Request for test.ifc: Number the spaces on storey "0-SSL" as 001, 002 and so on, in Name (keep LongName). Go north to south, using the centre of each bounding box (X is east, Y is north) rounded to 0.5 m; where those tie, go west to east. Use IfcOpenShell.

First a look at what the model holds.

```python
import ifcopenshell
import ifcopenshell.util.element
import ifcopenshell.util.placement

model = ifcopenshell.open("test.ifc")
print(model.schema)
storey = next(s for s in model.by_type("IfcBuildingStorey") if s.Name == "0-SSL")
spaces = [e for e in ifcopenshell.util.element.get_decomposition(storey) if e.is_a("IfcSpace")]
for e in sorted(spaces, key=lambda e: e.id()):
    origin = ifcopenshell.util.placement.get_local_placement(e.ObjectPlacement)[:3, 3]
    print(e.id(), e.Name, e.LongName, origin.round(2) + 0.0, sep=" | ")
```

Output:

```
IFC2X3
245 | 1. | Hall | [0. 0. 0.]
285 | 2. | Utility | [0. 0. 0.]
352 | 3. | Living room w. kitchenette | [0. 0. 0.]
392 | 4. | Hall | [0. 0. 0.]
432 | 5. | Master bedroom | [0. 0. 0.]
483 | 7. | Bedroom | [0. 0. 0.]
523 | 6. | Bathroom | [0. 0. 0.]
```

```python
import ifcopenshell
import ifcopenshell.geom
import ifcopenshell.util.element
import ifcopenshell.util.shape

model = ifcopenshell.open("test.ifc")
settings = ifcopenshell.geom.settings()
settings.set("use-world-coords", True)


def centre(element):
    shape = ifcopenshell.geom.create_shape(settings, element)
    return ifcopenshell.util.shape.get_bbox_centroid(shape.geometry)


storey = next(s for s in model.by_type("IfcBuildingStorey") if s.Name == "0-SSL")
spaces = [e for e in ifcopenshell.util.element.get_decomposition(storey) if e.is_a("IfcSpace")]

# Insertion points can sit at a corner or the storey origin, so sort by the geometry (in metres).
centres = {e: centre(e) for e in spaces}
spaces.sort(key=lambda e: (-round(centres[e][1] / 0.5), centres[e][0]))

for i, e in enumerate(spaces, start=1):
    number = f"0{i:02d}"
    e.Name = number
    print(e.id(), number)

model.write("test_updated.ifc")
```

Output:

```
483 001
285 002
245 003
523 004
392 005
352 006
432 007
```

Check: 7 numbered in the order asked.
